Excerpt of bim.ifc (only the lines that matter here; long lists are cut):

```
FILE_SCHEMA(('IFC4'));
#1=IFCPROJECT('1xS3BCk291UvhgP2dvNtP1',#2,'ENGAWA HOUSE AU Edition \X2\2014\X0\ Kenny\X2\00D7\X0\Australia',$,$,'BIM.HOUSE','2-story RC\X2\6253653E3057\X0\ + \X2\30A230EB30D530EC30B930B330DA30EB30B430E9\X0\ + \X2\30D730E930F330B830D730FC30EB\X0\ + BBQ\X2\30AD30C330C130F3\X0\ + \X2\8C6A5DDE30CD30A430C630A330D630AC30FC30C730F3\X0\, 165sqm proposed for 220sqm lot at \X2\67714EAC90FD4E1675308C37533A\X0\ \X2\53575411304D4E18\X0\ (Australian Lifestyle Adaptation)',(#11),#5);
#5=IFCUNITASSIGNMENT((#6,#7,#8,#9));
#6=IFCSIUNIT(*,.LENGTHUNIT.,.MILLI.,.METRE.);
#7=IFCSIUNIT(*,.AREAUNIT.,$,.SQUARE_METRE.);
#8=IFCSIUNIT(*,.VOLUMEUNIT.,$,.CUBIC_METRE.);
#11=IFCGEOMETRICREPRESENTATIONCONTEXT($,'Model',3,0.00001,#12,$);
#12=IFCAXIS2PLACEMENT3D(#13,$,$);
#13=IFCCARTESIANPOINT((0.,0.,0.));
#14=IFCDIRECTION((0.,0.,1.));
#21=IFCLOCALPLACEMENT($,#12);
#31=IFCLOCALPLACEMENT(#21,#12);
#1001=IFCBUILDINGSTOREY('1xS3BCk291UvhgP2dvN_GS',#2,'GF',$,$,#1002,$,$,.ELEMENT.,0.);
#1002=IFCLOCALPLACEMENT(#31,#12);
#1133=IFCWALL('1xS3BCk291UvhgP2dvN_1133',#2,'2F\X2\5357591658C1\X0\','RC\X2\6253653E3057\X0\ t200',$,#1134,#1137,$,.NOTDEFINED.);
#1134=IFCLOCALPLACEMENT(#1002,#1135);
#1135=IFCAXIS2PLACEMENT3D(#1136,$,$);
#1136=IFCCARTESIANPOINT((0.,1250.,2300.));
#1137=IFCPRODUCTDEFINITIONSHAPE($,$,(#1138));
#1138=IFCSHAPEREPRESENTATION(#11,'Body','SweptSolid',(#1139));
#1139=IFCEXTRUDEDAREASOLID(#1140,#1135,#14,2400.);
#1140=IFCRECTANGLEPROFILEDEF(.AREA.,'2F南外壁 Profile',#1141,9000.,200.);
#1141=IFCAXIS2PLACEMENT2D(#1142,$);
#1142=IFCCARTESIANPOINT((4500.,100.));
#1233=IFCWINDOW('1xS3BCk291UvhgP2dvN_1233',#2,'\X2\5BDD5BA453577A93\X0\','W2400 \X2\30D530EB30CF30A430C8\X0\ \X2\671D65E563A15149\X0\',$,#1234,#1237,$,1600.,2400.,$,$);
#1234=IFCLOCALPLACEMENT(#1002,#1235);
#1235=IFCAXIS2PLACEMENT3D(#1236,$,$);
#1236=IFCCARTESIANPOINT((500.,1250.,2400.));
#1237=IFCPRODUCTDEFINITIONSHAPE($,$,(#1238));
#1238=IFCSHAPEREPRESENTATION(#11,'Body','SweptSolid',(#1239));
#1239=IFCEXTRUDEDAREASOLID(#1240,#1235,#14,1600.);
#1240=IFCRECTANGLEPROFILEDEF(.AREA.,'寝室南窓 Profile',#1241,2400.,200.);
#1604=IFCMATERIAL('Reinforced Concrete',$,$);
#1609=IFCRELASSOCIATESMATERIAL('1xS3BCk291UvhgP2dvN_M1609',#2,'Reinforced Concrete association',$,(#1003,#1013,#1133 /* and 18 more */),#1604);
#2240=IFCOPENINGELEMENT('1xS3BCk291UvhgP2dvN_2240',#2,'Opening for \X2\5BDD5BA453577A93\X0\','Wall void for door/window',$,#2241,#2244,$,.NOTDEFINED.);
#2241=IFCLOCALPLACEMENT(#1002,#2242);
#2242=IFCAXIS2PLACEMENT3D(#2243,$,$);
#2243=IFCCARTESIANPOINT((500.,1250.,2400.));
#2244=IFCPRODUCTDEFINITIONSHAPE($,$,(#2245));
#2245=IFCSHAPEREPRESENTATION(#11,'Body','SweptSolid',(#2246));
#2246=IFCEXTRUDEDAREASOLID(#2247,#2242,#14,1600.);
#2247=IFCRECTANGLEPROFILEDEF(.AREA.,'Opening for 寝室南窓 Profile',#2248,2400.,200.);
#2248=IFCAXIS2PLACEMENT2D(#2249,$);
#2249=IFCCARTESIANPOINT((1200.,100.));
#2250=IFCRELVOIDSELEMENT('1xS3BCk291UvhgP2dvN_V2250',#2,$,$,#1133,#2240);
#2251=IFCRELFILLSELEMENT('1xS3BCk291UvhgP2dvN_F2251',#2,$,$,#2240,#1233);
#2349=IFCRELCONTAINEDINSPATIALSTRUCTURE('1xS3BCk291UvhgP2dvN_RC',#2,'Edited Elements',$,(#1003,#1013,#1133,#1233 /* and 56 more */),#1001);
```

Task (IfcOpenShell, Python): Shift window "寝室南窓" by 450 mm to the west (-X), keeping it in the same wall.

```python
import ifcopenshell
import ifcopenshell.api.geometry
import ifcopenshell.util.placement

model = ifcopenshell.open("bim.ifc")

window = model.by_guid("1xS3BCk291UvhgP2dvN_1233")
opening = window.FillsVoids[0].RelatingOpeningElement
wall = opening.VoidsElements[0].RelatingBuildingElement

wall_matrix = ifcopenshell.util.placement.get_local_placement(wall.ObjectPlacement)
shift = wall_matrix[:3, 0] * -450.0
before = ifcopenshell.util.placement.get_local_placement(window.ObjectPlacement)[:3, 3].copy()

# The window is not placed relative to its opening, so move both.
for product in (opening, window):
    matrix = ifcopenshell.util.placement.get_local_placement(product.ObjectPlacement)
    matrix[:3, 3] += shift
    ifcopenshell.api.geometry.edit_object_placement(model, product=product, matrix=matrix, is_si=False)

after = ifcopenshell.util.placement.get_local_placement(window.ObjectPlacement)[:3, 3]
print("window moved by", (after - before).round(3) + 0.0)

model.write("bim_rev.ifc")
```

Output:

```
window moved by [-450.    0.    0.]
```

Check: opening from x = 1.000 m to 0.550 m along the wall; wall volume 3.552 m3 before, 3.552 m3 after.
